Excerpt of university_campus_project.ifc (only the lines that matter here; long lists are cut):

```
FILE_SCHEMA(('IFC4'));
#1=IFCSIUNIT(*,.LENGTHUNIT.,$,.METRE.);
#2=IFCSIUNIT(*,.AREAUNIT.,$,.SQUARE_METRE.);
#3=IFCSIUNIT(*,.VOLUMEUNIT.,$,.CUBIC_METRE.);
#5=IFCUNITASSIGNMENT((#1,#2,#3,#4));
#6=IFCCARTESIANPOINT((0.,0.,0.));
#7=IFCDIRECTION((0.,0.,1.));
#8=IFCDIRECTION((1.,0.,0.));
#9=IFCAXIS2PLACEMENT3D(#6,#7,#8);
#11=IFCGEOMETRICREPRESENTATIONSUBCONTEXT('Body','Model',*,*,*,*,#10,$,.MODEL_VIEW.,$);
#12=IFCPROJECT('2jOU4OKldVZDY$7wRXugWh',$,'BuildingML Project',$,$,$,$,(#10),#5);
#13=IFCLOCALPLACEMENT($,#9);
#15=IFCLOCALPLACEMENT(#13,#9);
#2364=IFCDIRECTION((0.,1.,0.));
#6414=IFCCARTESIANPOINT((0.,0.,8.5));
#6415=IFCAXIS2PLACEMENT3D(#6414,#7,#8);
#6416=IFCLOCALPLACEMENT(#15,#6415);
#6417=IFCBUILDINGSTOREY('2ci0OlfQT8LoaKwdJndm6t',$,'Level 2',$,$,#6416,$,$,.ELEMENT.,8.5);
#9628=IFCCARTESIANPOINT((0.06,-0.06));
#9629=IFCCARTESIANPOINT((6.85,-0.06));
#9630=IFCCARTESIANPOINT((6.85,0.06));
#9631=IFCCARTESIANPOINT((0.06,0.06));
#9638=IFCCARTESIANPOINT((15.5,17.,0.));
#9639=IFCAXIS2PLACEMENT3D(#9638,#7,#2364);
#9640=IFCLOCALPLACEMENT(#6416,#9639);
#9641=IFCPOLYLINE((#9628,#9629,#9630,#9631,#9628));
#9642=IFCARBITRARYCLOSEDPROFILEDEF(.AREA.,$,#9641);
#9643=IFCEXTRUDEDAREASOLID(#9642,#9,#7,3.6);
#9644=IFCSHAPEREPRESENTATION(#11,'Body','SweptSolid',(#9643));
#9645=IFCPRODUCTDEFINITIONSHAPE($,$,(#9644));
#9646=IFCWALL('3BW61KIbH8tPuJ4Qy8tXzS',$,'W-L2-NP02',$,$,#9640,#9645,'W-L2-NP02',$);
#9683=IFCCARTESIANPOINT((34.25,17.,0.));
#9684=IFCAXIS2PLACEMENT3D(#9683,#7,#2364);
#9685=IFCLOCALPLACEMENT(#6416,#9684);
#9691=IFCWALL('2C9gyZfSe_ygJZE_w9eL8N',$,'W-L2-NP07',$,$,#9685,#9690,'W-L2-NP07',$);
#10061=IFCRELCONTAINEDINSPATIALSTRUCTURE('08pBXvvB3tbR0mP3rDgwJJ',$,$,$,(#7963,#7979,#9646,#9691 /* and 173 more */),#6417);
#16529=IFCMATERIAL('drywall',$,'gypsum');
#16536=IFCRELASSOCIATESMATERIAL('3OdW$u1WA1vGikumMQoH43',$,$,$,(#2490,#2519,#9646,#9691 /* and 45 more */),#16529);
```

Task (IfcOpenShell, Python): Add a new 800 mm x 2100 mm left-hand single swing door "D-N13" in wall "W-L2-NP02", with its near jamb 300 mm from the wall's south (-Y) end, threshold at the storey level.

```python
import numpy as np
import ifcopenshell
import ifcopenshell.api.feature
import ifcopenshell.api.geometry
import ifcopenshell.api.root
import ifcopenshell.api.spatial
import ifcopenshell.geom
import ifcopenshell.util.element
import ifcopenshell.util.placement
import ifcopenshell.util.representation
import ifcopenshell.util.shape
import ifcopenshell.util.unit

model = ifcopenshell.open("university_campus_project.ifc")
unit_scale = ifcopenshell.util.unit.calculate_unit_scale(model)
settings = ifcopenshell.geom.settings()


def volume(element):
    """Net volume in cubic metres, openings subtracted."""
    shape = ifcopenshell.geom.create_shape(settings, element)
    return ifcopenshell.util.shape.get_volume(shape.geometry)


wall = model.by_id(9646)
storey = ifcopenshell.util.element.get_container(wall, ifc_class="IfcBuildingStorey")
context = ifcopenshell.util.representation.get_context(model, "Model", "Body", "MODEL_VIEW")
before = volume(wall)

width, height, from_end, sill = 0.8, 2.1, 0.3, 0.0  # metres

# The wall runs along its own X axis, and the end named is its -X end.
wall_shape = ifcopenshell.geom.create_shape(settings, wall)
x, y, z = ifcopenshell.util.shape.get_vertices(wall_shape.geometry).T
start = x.min() + from_end
face, thickness = float(y.min()), float(y.max() - y.min())
wall_matrix = ifcopenshell.util.placement.get_local_placement(wall.ObjectPlacement)
level = ifcopenshell.util.placement.get_local_placement(storey.ObjectPlacement)[2, 3]


def in_wall(x, y):
    """Placement at x, y metres in the wall's axes, at sill height."""
    matrix = wall_matrix.copy()
    matrix[:, 3] = wall_matrix @ np.array([x / unit_scale, y / unit_scale, 0.0, 1.0])
    matrix[2, 3] = level + sill / unit_scale
    return matrix


# Opening: a box that overshoots both wall faces by 50 mm.
opening = ifcopenshell.api.root.create_entity(model, ifc_class="IfcOpeningElement", predefined_type="OPENING")
box = ifcopenshell.api.geometry.add_wall_representation(
    model, context=context, length=width, height=height, thickness=thickness + 0.1
)
ifcopenshell.api.geometry.assign_representation(model, product=opening, representation=box)
ifcopenshell.api.geometry.edit_object_placement(model, product=opening, matrix=in_wall(start, face - 0.05), is_si=False)
ifcopenshell.api.feature.add_feature(model, feature=opening, element=wall)

door = ifcopenshell.api.root.create_entity(model, ifc_class="IfcDoor", name="D-N13", predefined_type="DOOR")
door.OverallWidth, door.OverallHeight = width / unit_scale, height / unit_scale
door.OperationType = "SINGLE_SWING_LEFT"
body = ifcopenshell.api.geometry.add_door_representation(
    model,
    context=context,
    overall_width=door.OverallWidth,
    overall_height=door.OverallHeight,
    operation_type="SINGLE_SWING_LEFT",
    lining_properties={"LiningDepth": thickness / unit_scale, "ThresholdDepth": thickness / unit_scale},
)
ifcopenshell.api.geometry.assign_representation(model, product=door, representation=body)
ifcopenshell.api.spatial.assign_container(model, products=[door], relating_structure=storey)
ifcopenshell.api.feature.add_filling(model, opening=opening, element=door)

# The lining spans the wall, so the door starts at the wall face.
ifcopenshell.api.geometry.edit_object_placement(model, product=door, matrix=in_wall(start, face), is_si=False)

after = volume(wall)

print(f"wall volume {before:.3f} -> {after:.3f} m3")

model.write("university_campus_project_edited.ifc")
```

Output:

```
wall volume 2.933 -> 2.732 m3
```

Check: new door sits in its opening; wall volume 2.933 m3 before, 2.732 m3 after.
